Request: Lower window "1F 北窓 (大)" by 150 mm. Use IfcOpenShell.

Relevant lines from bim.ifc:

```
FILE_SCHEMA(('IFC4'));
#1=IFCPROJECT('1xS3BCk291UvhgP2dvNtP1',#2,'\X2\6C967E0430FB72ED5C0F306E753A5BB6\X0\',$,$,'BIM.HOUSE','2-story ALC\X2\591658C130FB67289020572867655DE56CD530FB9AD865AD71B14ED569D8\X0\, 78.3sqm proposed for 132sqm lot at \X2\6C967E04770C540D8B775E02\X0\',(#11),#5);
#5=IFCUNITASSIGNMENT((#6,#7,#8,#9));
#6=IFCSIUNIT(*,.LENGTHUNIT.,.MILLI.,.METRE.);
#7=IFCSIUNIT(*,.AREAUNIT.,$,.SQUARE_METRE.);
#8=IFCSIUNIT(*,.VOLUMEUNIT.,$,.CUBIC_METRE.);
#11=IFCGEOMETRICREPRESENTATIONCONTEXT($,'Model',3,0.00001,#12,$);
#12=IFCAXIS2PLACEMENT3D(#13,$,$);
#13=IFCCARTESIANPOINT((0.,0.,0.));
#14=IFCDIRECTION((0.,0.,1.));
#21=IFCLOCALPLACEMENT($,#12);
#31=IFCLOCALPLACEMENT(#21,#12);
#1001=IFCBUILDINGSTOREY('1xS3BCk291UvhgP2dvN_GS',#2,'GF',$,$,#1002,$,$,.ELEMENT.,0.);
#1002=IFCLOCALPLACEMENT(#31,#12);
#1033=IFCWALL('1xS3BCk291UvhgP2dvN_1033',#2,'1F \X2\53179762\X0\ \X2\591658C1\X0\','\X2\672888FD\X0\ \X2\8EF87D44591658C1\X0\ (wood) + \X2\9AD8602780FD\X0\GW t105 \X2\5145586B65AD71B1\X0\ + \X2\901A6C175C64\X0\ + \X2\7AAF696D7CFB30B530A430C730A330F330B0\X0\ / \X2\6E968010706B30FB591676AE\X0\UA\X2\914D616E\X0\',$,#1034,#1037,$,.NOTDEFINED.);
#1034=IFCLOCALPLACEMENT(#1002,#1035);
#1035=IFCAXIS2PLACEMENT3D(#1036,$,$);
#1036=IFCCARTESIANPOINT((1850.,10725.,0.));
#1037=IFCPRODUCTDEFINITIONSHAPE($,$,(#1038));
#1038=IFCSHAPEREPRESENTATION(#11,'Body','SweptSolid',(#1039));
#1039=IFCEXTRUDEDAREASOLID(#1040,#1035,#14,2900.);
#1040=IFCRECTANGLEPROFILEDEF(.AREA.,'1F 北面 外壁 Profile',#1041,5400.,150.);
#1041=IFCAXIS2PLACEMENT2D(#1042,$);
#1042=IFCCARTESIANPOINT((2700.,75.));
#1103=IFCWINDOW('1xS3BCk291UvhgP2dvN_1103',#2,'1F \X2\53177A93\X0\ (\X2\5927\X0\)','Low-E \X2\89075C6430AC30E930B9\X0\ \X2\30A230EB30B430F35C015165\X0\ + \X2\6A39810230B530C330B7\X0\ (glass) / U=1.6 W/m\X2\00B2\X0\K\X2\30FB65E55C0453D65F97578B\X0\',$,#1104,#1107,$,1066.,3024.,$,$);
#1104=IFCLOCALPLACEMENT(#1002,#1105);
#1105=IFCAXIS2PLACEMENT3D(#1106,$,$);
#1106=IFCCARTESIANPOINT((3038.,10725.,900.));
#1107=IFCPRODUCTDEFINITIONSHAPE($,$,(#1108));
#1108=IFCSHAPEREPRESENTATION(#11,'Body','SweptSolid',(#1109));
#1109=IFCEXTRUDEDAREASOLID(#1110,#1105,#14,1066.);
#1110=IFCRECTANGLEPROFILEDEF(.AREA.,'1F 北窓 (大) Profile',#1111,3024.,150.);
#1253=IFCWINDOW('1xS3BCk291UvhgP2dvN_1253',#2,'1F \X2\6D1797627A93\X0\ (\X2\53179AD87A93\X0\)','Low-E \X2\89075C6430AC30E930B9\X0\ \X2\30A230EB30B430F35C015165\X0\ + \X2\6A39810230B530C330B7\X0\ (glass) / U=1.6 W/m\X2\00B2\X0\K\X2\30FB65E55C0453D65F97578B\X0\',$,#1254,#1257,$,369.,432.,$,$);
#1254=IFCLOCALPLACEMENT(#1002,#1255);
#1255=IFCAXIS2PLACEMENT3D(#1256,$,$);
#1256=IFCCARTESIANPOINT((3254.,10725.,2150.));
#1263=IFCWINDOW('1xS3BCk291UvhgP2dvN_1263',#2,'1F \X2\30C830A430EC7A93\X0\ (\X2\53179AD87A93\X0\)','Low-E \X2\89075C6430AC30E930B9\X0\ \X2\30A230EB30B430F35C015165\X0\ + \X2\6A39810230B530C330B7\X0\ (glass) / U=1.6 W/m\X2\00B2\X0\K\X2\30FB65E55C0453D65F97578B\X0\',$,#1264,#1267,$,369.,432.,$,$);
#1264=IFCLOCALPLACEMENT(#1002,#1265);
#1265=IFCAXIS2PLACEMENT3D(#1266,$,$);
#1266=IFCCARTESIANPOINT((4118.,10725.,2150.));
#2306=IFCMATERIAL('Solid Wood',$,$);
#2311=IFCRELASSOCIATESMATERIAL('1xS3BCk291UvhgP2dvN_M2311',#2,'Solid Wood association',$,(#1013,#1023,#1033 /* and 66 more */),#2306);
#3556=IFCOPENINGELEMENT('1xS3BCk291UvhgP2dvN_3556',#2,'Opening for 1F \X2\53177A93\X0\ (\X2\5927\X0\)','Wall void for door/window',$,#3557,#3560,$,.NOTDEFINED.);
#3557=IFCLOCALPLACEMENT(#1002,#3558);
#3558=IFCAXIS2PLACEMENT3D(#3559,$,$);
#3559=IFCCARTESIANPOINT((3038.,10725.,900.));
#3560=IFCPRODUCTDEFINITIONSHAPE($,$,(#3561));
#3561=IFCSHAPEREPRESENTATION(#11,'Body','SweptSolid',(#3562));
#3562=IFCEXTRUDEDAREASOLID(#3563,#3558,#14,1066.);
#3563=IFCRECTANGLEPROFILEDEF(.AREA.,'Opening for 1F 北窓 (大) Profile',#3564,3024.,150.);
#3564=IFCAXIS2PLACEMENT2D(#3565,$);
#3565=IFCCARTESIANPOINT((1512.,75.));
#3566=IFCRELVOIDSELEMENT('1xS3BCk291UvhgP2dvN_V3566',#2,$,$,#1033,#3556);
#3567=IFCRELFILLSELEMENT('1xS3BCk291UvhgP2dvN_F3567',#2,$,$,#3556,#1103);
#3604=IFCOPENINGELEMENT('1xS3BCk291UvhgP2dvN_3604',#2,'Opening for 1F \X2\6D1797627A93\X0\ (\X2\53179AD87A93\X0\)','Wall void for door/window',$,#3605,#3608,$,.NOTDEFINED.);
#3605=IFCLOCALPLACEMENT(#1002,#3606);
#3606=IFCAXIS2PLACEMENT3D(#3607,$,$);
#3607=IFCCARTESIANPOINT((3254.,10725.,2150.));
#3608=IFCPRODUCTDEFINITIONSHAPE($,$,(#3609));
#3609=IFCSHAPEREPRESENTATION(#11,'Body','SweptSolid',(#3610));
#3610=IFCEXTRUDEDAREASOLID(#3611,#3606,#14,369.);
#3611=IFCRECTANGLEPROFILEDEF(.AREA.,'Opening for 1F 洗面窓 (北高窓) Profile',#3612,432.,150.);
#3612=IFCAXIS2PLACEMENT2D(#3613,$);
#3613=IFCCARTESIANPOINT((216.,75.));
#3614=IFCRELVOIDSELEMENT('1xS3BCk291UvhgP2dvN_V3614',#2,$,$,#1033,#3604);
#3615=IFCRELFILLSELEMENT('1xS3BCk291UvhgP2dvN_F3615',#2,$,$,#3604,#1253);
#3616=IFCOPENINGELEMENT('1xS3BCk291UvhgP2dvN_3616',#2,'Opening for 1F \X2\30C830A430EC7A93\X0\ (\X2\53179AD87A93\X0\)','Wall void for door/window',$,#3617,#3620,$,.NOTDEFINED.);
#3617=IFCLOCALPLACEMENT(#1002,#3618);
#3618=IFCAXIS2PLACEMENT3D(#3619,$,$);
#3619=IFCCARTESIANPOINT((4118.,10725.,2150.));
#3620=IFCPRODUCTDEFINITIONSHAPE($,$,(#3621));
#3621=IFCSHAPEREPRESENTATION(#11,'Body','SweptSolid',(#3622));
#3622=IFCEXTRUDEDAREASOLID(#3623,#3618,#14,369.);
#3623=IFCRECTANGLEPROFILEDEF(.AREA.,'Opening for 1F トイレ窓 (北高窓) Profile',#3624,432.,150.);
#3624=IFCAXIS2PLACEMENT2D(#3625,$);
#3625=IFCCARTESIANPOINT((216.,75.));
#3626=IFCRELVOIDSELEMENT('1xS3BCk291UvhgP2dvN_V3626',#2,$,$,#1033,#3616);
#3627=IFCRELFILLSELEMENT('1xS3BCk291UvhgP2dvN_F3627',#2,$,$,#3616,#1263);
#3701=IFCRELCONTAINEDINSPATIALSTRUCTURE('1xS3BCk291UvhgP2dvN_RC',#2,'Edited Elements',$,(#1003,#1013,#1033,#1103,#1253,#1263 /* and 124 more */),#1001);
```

```python
import numpy as np
import ifcopenshell
import ifcopenshell.api.geometry
import ifcopenshell.util.placement
import ifcopenshell.util.unit

model = ifcopenshell.open("bim.ifc")
unit_scale = ifcopenshell.util.unit.calculate_unit_scale(model)

window = model.by_id(1103)
opening = window.FillsVoids[0].RelatingOpeningElement
dz = -150.0

shift = np.array([0.0, 0.0, dz])
# The window is not placed relative to its opening, so move both.
for product in (opening, window):
    matrix = ifcopenshell.util.placement.get_local_placement(product.ObjectPlacement)
    matrix[:3, 3] += shift
    ifcopenshell.api.geometry.edit_object_placement(model, product=product, matrix=matrix, is_si=False)

print(f"moved by {dz * unit_scale:+.3f} m")

model.write("bim_updated.ifc")
```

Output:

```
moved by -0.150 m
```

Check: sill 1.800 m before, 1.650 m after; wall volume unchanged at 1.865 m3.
